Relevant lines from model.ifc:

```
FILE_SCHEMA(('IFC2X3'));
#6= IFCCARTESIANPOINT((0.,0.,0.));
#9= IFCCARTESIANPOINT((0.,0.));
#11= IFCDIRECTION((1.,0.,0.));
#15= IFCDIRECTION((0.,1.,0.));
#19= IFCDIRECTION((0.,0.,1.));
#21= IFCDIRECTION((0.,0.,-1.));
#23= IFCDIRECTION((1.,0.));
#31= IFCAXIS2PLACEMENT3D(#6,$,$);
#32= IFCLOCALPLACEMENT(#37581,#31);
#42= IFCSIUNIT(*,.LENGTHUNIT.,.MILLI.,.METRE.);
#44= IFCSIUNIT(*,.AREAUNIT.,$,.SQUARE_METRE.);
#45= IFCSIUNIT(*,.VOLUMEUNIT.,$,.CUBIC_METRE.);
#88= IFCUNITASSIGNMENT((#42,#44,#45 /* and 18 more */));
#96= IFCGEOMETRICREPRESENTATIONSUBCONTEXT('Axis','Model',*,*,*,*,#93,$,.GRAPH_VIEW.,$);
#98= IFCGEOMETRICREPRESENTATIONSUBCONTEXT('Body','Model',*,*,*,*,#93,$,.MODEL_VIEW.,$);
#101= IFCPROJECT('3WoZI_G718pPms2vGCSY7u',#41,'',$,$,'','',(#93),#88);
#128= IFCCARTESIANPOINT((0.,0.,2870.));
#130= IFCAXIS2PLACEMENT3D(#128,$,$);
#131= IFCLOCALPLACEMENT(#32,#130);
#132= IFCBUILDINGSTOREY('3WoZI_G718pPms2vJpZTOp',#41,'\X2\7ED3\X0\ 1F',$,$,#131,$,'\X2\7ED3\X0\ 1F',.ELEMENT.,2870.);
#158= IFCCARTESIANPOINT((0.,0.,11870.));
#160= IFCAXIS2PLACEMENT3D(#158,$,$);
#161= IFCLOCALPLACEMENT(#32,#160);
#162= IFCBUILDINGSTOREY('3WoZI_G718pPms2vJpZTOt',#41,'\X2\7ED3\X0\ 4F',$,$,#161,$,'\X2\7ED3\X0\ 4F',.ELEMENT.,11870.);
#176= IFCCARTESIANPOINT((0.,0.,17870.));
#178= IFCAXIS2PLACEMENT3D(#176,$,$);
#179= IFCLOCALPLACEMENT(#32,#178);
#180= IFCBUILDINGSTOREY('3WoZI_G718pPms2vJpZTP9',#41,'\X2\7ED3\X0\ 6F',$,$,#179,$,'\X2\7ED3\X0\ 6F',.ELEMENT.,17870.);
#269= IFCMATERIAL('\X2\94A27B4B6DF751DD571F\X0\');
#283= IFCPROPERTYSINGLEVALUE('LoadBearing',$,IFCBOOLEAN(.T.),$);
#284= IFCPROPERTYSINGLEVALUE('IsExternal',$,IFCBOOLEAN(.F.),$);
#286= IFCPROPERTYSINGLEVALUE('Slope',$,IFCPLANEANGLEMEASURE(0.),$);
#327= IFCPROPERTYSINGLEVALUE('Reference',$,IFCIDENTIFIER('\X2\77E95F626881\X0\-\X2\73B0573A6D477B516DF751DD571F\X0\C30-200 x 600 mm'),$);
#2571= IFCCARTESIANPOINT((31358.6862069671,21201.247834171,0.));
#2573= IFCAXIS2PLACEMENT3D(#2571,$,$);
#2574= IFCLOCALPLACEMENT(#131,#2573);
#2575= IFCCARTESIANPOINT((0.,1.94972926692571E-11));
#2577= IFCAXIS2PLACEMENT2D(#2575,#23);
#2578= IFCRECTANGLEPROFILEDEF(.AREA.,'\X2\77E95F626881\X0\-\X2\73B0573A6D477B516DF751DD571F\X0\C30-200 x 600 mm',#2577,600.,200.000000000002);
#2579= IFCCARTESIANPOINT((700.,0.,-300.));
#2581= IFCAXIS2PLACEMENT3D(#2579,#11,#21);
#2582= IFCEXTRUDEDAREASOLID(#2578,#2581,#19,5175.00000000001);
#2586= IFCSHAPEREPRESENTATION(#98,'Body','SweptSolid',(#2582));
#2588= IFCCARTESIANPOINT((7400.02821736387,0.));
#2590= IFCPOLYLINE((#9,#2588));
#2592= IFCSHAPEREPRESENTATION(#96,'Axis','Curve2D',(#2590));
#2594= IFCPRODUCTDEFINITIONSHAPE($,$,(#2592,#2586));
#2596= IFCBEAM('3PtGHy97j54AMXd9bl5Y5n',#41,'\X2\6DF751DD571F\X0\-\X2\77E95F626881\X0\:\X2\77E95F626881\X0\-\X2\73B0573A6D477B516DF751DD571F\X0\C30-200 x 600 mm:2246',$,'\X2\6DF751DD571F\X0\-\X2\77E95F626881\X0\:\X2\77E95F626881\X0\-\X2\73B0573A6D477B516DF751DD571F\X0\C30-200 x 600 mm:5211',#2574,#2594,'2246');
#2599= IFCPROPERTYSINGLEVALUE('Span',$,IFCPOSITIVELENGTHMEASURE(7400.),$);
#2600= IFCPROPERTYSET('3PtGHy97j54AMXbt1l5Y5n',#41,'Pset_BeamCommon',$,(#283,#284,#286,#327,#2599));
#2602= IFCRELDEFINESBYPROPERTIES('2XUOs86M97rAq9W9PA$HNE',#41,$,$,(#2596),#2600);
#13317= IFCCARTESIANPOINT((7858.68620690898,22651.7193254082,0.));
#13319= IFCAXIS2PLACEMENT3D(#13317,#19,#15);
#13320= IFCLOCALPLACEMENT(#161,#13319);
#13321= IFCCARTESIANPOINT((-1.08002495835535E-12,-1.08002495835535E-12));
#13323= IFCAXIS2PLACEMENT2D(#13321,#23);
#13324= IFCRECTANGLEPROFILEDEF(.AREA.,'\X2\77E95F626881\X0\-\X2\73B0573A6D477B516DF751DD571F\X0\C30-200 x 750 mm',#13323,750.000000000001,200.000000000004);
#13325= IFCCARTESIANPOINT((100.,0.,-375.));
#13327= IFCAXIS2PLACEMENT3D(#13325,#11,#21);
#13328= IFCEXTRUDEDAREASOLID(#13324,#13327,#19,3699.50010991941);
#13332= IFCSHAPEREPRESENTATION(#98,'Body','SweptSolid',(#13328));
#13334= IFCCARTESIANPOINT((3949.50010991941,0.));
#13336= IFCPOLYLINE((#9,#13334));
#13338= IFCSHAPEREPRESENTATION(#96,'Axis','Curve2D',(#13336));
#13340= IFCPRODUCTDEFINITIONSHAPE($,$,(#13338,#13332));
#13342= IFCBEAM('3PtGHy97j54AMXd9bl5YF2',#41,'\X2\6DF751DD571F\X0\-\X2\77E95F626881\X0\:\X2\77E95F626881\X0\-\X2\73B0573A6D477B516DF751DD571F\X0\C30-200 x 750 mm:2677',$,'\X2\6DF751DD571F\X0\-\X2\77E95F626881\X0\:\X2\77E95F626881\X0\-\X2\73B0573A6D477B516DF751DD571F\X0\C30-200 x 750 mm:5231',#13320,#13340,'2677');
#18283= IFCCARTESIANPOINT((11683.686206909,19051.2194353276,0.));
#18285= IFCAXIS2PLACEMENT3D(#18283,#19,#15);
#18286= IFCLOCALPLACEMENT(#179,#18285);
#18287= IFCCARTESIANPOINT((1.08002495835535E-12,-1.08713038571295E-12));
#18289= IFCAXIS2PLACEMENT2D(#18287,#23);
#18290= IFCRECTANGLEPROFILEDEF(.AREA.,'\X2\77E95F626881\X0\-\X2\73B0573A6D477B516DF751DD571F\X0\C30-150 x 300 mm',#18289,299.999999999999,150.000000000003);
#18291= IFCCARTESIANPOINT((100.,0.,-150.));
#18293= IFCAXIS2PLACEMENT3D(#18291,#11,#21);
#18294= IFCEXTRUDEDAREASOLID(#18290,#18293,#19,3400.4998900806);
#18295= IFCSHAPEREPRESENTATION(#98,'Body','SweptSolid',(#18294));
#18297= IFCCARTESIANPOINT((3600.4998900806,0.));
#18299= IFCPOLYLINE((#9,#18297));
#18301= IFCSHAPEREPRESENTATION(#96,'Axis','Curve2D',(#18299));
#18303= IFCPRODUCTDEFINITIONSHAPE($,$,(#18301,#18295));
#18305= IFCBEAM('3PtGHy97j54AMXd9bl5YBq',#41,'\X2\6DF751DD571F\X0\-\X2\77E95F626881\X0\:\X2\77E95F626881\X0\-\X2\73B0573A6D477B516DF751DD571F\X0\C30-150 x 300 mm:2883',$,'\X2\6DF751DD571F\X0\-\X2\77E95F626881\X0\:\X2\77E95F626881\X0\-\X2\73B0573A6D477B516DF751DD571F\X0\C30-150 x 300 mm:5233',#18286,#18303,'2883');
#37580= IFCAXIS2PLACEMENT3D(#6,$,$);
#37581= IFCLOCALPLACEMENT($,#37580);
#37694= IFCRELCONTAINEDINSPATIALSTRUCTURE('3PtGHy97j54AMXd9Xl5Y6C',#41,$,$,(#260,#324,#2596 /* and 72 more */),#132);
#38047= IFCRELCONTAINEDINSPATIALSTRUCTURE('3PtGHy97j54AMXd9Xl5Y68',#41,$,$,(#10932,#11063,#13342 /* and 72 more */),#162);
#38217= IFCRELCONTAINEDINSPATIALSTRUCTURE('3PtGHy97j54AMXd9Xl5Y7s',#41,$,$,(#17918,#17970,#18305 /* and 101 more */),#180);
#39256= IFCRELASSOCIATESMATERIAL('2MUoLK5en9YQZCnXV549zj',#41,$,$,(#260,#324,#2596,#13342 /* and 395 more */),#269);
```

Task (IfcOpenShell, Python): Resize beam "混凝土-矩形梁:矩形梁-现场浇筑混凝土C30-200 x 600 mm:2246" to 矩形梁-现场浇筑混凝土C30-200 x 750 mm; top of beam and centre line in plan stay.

```python
import ifcopenshell
import ifcopenshell.api.pset
import ifcopenshell.util.element
import ifcopenshell.util.representation

model = ifcopenshell.open("model.ifc")

member = model.by_guid("3PtGHy97j54AMXd9bl5Y5n")
source = next(p for p in model.by_type("IfcRectangleProfileDef") if p.ProfileName == "矩形梁-现场浇筑混凝土C30-200 x 750 mm")

body = ifcopenshell.util.representation.get_representation(member, "Model", "Body")
solid = body.Items[0]
old_profile = solid.SweptArea

# Copy the section's sizes but keep this member's own profile position.
profile = ifcopenshell.util.element.copy(model, source)
# Profiles are centred, so shift by half the change in depth to hold the top.
shift = (old_profile.XDim - profile.XDim) / 2
x, y = old_profile.Position.Location.Coordinates
up = (-1.0, 0.0)  # upwards, in the solid's own plane
location = model.createIfcCartesianPoint((x + up[0] * shift, y + up[1] * shift))
profile.Position = model.createIfcAxis2Placement2D(location, old_profile.Position.RefDirection)
solid.SweptArea = profile
if not model.get_total_inverses(old_profile):
    ifcopenshell.util.element.remove_deep2(model, old_profile)
member.Name = member.Name.replace("矩形梁-现场浇筑混凝土C30-200 x 600 mm", "矩形梁-现场浇筑混凝土C30-200 x 750 mm")
member.ObjectType = member.ObjectType.replace("矩形梁-现场浇筑混凝土C30-200 x 600 mm", "矩形梁-现场浇筑混凝土C30-200 x 750 mm")
pset = model.by_id(ifcopenshell.util.element.get_pset(member, "Pset_BeamCommon", should_inherit=False)["id"])
ifcopenshell.api.pset.edit_pset(model, pset=pset, properties={"Reference": "矩形梁-现场浇筑混凝土C30-200 x 750 mm"})

print(solid.SweptArea)

model.write("model_updated.ifc")
```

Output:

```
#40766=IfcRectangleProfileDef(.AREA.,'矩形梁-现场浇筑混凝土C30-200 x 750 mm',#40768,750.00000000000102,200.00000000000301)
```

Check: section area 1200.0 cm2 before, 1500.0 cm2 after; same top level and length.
